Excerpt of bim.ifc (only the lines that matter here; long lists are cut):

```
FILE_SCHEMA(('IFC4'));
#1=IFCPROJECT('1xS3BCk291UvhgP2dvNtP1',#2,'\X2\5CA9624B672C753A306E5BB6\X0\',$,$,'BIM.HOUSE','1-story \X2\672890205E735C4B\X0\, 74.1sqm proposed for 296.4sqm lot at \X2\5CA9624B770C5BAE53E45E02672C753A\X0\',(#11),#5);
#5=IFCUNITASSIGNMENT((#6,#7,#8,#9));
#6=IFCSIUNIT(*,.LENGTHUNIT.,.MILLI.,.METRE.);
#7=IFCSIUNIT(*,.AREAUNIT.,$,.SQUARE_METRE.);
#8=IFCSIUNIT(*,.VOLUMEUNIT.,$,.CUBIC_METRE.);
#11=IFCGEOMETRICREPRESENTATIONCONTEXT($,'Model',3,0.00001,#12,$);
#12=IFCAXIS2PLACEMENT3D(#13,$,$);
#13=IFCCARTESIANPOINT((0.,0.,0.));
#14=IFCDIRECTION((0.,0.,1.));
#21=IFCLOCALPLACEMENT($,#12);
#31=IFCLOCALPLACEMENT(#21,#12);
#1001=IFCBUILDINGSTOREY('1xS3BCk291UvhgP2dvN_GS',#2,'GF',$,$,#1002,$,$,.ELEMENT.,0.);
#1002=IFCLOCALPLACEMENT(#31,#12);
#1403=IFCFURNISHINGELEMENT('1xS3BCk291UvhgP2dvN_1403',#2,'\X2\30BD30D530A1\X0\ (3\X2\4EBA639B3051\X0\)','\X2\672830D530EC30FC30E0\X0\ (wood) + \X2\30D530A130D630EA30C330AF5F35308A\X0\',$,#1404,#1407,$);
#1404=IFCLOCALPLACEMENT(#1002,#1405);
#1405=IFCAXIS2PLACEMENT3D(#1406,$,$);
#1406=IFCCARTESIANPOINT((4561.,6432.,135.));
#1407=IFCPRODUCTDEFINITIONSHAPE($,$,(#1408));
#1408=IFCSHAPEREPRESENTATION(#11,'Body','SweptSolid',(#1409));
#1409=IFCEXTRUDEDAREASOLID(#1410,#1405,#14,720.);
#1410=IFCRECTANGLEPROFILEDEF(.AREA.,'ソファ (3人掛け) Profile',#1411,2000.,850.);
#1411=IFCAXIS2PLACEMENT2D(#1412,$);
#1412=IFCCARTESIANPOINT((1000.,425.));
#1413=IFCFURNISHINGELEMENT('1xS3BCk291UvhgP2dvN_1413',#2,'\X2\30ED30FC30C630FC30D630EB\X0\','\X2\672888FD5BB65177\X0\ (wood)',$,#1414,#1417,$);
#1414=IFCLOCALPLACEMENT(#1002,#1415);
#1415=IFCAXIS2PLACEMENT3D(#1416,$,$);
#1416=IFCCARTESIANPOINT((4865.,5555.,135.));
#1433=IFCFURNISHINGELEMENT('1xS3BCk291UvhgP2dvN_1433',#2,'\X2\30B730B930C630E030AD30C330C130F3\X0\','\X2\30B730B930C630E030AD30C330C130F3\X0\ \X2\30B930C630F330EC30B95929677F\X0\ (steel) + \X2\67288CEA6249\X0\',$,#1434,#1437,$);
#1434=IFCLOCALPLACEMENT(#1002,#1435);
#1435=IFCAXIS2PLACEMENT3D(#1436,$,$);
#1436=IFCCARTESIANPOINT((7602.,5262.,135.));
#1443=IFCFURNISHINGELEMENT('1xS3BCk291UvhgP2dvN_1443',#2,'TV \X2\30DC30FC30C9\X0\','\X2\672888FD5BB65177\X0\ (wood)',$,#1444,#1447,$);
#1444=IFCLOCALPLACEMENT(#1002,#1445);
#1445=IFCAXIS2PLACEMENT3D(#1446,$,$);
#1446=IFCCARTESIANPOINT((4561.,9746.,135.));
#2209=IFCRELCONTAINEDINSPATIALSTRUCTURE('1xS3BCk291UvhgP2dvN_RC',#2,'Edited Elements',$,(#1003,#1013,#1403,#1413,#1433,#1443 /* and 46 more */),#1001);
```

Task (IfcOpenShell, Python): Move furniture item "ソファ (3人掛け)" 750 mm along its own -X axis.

```python
import ifcopenshell
import ifcopenshell.api.geometry
import ifcopenshell.util.placement

model = ifcopenshell.open("bim.ifc")

item = model.by_id(1403)
matrix = ifcopenshell.util.placement.get_local_placement(item.ObjectPlacement)
matrix[:3, 3] -= matrix[:3, 0] * 750.0
ifcopenshell.api.geometry.edit_object_placement(model, product=item, matrix=matrix, is_si=False)

print(ifcopenshell.util.placement.get_local_placement(item.ObjectPlacement).round(3) + 0.0)

model.write("bim_edited.ifc")
```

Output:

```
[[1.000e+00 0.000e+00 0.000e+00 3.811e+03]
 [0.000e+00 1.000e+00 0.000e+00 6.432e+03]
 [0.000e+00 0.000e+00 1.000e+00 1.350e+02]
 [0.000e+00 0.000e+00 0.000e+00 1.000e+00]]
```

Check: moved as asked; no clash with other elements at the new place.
